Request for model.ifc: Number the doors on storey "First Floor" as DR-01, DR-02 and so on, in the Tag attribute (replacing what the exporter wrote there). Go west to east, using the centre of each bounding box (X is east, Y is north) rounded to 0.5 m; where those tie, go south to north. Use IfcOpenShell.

First a look at what the model holds.

```python
import ifcopenshell
import ifcopenshell.util.element
import ifcopenshell.util.placement

model = ifcopenshell.open("model.ifc")
print(model.schema)
storey = next(s for s in model.by_type("IfcBuildingStorey") if s.Name == "First Floor")
doors = [e for e in ifcopenshell.util.element.get_decomposition(storey) if e.is_a("IfcDoor")]
for e in sorted(doors, key=lambda e: e.id()):
    origin = ifcopenshell.util.placement.get_local_placement(e.ObjectPlacement)[:3, 3]
    print(e.id(), e.Tag, e.Name, origin.round(2) + 0.0, sep=" | ")
```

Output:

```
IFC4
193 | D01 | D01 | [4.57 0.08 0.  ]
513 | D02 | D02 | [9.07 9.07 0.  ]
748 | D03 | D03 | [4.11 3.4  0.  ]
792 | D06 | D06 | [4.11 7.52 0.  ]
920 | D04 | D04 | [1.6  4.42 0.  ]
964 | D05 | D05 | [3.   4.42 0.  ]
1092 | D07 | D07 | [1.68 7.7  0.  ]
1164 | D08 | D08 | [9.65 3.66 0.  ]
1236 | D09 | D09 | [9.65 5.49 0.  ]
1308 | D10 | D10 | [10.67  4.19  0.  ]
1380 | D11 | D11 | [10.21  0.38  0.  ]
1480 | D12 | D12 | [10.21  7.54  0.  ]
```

```python
import ifcopenshell
import ifcopenshell.geom
import ifcopenshell.util.element
import ifcopenshell.util.shape

model = ifcopenshell.open("model.ifc")
settings = ifcopenshell.geom.settings()
settings.set("use-world-coords", True)


def centre(element):
    shape = ifcopenshell.geom.create_shape(settings, element)
    return ifcopenshell.util.shape.get_bbox_centroid(shape.geometry)


storey = next(s for s in model.by_type("IfcBuildingStorey") if s.Name == "First Floor")
doors = [e for e in ifcopenshell.util.element.get_decomposition(storey) if e.is_a("IfcDoor")]

# Insertion points can sit at a corner or the storey origin, so sort by the geometry (in metres).
centres = {e: centre(e) for e in doors}
doors.sort(key=lambda e: (round(centres[e][0] / 0.5), centres[e][1]))

for i, e in enumerate(doors, start=1):
    number = f"DR-{i:02d}"
    e.Tag = number
    print(e.id(), number)

model.write("model_edited.ifc")
```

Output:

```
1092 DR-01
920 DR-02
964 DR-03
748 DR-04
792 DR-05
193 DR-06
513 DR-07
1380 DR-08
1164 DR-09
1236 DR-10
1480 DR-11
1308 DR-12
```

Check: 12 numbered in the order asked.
